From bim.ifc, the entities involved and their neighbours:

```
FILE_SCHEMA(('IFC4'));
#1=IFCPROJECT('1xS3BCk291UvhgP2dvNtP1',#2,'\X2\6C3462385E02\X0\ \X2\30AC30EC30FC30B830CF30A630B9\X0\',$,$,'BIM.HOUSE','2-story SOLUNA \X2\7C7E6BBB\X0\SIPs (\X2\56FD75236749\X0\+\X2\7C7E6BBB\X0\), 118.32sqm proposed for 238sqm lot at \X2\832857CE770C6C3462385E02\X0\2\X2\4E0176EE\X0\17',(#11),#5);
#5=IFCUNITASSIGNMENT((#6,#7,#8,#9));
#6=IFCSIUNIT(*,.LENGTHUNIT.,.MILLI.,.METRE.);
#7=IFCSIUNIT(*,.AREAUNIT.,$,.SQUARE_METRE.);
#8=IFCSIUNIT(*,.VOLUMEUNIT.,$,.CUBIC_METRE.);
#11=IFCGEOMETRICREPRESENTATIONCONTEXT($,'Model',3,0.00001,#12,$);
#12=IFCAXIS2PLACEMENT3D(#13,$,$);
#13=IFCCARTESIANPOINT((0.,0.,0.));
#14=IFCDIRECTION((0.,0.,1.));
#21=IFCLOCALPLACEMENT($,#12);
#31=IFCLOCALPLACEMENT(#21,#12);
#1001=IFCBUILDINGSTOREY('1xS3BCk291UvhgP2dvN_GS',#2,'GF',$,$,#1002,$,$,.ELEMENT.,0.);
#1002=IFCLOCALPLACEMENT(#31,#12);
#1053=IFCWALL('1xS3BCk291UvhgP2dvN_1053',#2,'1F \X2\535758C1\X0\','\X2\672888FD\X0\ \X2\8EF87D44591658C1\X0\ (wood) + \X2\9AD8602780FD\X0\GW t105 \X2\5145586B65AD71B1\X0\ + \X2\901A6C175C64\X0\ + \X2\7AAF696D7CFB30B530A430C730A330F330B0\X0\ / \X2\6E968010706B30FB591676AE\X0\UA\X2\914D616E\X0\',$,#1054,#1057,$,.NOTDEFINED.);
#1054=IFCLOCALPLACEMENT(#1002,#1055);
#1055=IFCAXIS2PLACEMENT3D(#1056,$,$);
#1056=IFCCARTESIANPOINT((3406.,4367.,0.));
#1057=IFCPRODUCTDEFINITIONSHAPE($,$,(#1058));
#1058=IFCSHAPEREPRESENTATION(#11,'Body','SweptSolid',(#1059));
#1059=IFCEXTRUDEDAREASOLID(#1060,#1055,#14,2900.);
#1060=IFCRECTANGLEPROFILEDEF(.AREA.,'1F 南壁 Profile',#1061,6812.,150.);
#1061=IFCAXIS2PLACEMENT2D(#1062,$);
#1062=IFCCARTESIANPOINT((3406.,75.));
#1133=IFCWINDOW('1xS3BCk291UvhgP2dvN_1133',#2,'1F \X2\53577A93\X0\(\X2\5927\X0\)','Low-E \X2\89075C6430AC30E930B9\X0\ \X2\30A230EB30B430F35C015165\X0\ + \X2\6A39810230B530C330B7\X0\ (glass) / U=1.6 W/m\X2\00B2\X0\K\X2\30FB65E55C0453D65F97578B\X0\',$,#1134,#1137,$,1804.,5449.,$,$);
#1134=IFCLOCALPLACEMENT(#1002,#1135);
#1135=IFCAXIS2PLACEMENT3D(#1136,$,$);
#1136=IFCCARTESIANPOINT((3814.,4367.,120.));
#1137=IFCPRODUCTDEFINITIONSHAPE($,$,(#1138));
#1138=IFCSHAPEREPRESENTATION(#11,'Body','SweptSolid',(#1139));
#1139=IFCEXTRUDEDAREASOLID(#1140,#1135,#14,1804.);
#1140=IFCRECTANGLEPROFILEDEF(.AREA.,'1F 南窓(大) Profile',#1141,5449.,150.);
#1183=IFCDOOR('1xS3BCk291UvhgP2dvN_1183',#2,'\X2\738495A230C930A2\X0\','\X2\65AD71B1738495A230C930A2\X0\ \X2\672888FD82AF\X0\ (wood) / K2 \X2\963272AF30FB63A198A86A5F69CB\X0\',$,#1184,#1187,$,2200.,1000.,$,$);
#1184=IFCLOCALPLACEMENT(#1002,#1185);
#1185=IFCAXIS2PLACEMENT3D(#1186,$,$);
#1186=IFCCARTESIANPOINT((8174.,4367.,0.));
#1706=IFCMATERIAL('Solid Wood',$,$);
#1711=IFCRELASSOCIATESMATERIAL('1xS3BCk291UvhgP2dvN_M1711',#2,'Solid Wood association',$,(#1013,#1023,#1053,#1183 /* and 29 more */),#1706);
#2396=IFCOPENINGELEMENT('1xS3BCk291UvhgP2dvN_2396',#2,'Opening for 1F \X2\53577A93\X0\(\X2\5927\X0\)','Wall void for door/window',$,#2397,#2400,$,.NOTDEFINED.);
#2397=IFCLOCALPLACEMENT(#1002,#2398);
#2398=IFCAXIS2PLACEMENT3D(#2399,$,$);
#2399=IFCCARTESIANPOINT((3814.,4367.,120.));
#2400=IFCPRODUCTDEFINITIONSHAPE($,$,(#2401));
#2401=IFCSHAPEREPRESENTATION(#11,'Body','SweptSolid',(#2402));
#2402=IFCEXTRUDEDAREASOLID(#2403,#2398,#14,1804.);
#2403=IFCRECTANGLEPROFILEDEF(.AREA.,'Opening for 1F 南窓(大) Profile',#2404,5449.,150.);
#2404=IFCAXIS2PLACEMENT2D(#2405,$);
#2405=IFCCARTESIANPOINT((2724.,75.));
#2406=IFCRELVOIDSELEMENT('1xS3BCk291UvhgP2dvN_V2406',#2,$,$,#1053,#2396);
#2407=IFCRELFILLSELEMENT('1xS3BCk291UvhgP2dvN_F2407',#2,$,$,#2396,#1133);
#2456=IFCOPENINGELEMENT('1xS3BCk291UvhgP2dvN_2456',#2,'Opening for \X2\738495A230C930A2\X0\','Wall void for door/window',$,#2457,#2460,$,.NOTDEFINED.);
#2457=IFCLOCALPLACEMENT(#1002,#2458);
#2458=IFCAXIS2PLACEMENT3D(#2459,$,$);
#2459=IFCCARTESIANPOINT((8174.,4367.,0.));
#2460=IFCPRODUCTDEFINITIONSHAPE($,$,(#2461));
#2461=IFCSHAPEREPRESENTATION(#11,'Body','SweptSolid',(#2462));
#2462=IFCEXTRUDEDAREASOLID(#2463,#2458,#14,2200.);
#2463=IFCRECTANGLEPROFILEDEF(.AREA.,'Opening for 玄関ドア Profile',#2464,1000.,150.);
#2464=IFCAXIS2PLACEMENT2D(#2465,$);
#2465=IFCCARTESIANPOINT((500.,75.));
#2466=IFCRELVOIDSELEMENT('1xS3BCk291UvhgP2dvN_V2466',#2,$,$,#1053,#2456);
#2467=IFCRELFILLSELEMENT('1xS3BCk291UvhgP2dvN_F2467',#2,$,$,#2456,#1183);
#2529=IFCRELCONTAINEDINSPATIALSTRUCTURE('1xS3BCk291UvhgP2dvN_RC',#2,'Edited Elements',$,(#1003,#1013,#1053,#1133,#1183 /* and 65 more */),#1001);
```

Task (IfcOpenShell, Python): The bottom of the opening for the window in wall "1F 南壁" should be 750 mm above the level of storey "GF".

```python
import numpy as np
import ifcopenshell
import ifcopenshell.api.geometry
import ifcopenshell.geom
import ifcopenshell.util.element
import ifcopenshell.util.placement
import ifcopenshell.util.shape
import ifcopenshell.util.unit

model = ifcopenshell.open("bim.ifc")
unit_scale = ifcopenshell.util.unit.calculate_unit_scale(model)

window = model.by_guid("1xS3BCk291UvhgP2dvN_1133")
opening = window.FillsVoids[0].RelatingOpeningElement
storey = ifcopenshell.util.element.get_container(window, ifc_class="IfcBuildingStorey")
level = ifcopenshell.util.placement.get_local_placement(storey.ObjectPlacement)[2, 3]

# The opening's origin need not be at the sill, so measure its lowest point.
shape = ifcopenshell.geom.create_shape(ifcopenshell.geom.settings(), opening)
bottom = ifcopenshell.util.shape.get_shape_bottom_elevation(shape, shape.geometry) / unit_scale
dz = level + 0.75 / unit_scale - bottom

shift = np.array([0.0, 0.0, dz])
# The window is not placed relative to its opening, so move both.
for product in (opening, window):
    matrix = ifcopenshell.util.placement.get_local_placement(product.ObjectPlacement)
    matrix[:3, 3] += shift
    ifcopenshell.api.geometry.edit_object_placement(model, product=product, matrix=matrix, is_si=False)

print(f"moved by {dz * unit_scale:+.3f} m")

model.write("bim_edited.ifc")
```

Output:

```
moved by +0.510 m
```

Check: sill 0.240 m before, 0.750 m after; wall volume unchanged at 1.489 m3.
